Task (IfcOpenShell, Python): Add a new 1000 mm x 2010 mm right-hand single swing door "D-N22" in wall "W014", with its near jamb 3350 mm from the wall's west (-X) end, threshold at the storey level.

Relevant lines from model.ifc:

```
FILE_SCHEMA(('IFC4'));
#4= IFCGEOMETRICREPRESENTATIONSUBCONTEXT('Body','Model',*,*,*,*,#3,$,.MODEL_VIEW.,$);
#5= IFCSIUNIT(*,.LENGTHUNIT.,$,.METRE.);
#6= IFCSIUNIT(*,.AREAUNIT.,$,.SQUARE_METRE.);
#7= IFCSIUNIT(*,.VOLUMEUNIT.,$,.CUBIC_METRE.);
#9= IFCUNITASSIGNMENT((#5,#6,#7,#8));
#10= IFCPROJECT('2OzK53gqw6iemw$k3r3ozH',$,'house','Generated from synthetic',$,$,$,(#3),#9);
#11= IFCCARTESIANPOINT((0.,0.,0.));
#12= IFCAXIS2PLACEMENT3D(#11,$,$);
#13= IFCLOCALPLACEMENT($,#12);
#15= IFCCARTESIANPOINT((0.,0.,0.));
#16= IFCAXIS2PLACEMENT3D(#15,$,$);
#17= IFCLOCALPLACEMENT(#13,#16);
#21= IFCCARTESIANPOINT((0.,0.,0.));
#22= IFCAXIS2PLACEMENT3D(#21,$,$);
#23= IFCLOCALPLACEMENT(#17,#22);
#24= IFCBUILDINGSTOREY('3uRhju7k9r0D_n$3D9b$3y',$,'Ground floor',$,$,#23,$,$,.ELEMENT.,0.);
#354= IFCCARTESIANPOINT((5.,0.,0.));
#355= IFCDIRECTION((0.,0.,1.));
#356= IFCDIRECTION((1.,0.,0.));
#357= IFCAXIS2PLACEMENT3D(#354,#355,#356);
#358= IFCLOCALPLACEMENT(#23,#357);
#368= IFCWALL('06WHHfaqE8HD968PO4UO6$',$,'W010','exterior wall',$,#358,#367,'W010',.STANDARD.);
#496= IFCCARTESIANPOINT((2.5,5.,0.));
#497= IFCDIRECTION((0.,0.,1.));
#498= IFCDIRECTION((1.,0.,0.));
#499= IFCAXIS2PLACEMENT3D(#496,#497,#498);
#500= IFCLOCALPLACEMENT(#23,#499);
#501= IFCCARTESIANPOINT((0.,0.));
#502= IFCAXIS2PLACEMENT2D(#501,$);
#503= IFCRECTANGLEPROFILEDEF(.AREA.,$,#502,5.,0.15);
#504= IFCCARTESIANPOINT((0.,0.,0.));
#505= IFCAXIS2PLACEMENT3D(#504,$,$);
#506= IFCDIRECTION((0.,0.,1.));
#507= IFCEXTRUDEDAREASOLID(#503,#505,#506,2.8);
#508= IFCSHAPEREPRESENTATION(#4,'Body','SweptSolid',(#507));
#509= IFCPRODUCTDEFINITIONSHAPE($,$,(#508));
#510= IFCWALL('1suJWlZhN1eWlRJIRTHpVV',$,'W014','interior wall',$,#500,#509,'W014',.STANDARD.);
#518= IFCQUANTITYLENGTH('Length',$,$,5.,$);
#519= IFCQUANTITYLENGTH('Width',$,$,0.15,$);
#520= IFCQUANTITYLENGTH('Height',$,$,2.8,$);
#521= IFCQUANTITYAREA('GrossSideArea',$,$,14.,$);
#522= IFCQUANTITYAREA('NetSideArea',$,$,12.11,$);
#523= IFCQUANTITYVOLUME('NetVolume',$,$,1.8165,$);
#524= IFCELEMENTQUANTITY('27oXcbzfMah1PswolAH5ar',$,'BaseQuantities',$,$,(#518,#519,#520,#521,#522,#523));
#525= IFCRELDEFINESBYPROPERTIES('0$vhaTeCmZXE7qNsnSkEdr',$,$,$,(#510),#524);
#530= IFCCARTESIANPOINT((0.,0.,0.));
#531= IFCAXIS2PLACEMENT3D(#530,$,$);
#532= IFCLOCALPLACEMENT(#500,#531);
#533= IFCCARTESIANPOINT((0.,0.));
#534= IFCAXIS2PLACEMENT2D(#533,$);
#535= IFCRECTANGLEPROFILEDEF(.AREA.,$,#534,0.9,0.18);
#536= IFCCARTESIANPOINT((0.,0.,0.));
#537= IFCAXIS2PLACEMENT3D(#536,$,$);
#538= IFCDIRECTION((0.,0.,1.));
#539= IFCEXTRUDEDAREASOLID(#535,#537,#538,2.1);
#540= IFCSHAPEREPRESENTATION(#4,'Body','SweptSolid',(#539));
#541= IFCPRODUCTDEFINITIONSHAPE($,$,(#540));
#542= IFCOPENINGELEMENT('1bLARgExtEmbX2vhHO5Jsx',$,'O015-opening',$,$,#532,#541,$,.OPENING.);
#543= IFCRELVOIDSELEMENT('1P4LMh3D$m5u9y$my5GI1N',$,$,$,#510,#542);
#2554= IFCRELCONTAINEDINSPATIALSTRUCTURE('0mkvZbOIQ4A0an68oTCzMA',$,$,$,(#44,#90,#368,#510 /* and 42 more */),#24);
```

```python
import numpy as np
import ifcopenshell
import ifcopenshell.api.feature
import ifcopenshell.api.geometry
import ifcopenshell.api.pset
import ifcopenshell.api.root
import ifcopenshell.api.spatial
import ifcopenshell.geom
import ifcopenshell.util.element
import ifcopenshell.util.placement
import ifcopenshell.util.representation
import ifcopenshell.util.shape
import ifcopenshell.util.unit

model = ifcopenshell.open("model.ifc")
unit_scale = ifcopenshell.util.unit.calculate_unit_scale(model)
area_scale = ifcopenshell.util.unit.calculate_unit_scale(model, "AREAUNIT")
volume_scale = ifcopenshell.util.unit.calculate_unit_scale(model, "VOLUMEUNIT")
settings = ifcopenshell.geom.settings()


def volume(element):
    """Net volume in cubic metres, openings subtracted."""
    shape = ifcopenshell.geom.create_shape(settings, element)
    return ifcopenshell.util.shape.get_volume(shape.geometry)


wall = model.by_guid("1suJWlZhN1eWlRJIRTHpVV")
storey = ifcopenshell.util.element.get_container(wall, ifc_class="IfcBuildingStorey")
context = ifcopenshell.util.representation.get_context(model, "Model", "Body", "MODEL_VIEW")
before = volume(wall)

width, height, from_end, sill = 1, 2.01, 3.35, 0.0  # metres

# The wall runs along its own X axis, and the end named is its -X end.
wall_shape = ifcopenshell.geom.create_shape(settings, wall)
x, y, z = ifcopenshell.util.shape.get_vertices(wall_shape.geometry).T
start = x.min() + from_end
face, thickness = float(y.min()), float(y.max() - y.min())
wall_matrix = ifcopenshell.util.placement.get_local_placement(wall.ObjectPlacement)
level = ifcopenshell.util.placement.get_local_placement(storey.ObjectPlacement)[2, 3]


def in_wall(x, y):
    """Placement at x, y metres in the wall's axes, at sill height."""
    matrix = wall_matrix.copy()
    matrix[:, 3] = wall_matrix @ np.array([x / unit_scale, y / unit_scale, 0.0, 1.0])
    matrix[2, 3] = level + sill / unit_scale
    return matrix


# Opening: a box that overshoots both wall faces by 50 mm.
opening = ifcopenshell.api.root.create_entity(model, ifc_class="IfcOpeningElement", predefined_type="OPENING")
box = ifcopenshell.api.geometry.add_wall_representation(
    model, context=context, length=width, height=height, thickness=thickness + 0.1
)
ifcopenshell.api.geometry.assign_representation(model, product=opening, representation=box)
ifcopenshell.api.geometry.edit_object_placement(model, product=opening, matrix=in_wall(start, face - 0.05), is_si=False)
ifcopenshell.api.feature.add_feature(model, feature=opening, element=wall)

door = ifcopenshell.api.root.create_entity(model, ifc_class="IfcDoor", name="D-N22", predefined_type="DOOR")
door.OverallWidth, door.OverallHeight = width / unit_scale, height / unit_scale
door.OperationType = "SINGLE_SWING_RIGHT"
body = ifcopenshell.api.geometry.add_door_representation(
    model,
    context=context,
    overall_width=door.OverallWidth,
    overall_height=door.OverallHeight,
    operation_type="SINGLE_SWING_RIGHT",
    lining_properties={"LiningDepth": thickness / unit_scale, "ThresholdDepth": thickness / unit_scale},
)
ifcopenshell.api.geometry.assign_representation(model, product=door, representation=body)
ifcopenshell.api.spatial.assign_container(model, products=[door], relating_structure=storey)
ifcopenshell.api.feature.add_filling(model, opening=opening, element=door)

# The lining spans the wall, so the door starts at the wall face.
ifcopenshell.api.geometry.edit_object_placement(model, product=door, matrix=in_wall(start, face), is_si=False)

after = volume(wall)

# Update the wall's stored quantities.
qto = model.by_id(ifcopenshell.util.element.get_pset(wall, "BaseQuantities", should_inherit=False)["id"])
ifcopenshell.api.pset.edit_qto(model, qto=qto, properties={
    "NetSideArea": after / thickness / area_scale,
    "NetVolume": after / volume_scale,
})

print(f"wall volume {before:.3f} -> {after:.3f} m3")

model.write("model_edited.ifc")
```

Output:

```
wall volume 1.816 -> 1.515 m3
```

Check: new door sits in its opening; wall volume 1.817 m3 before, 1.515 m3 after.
